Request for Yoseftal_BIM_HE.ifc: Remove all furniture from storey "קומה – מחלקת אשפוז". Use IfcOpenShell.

First a look at what the model holds.

```python
import ifcopenshell
import ifcopenshell.util.element

model = ifcopenshell.open("Yoseftal_BIM_HE.ifc")
print(model.schema)
storey = next(s for s in model.by_type("IfcBuildingStorey") if s.Name == "קומה – מחלקת אשפוז")
furniture = [e for e in ifcopenshell.util.element.get_decomposition(storey) if e.is_a("IfcFurnishingElement")]
seen = {}
for e in furniture:
    element_type = ifcopenshell.util.element.get_type(e)
    name = element_type.Name if element_type not in (None, e) else None
    seen[name] = seen.get(name, 0) + 1
for name, count in sorted(seen.items(), key=str):
    print(count, "x", name)
```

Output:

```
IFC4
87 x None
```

```python
import ifcopenshell
import ifcopenshell.api.root
import ifcopenshell.util.element

model = ifcopenshell.open("Yoseftal_BIM_HE.ifc")

storey = next(s for s in model.by_type("IfcBuildingStorey") if s.Name == "קומה – מחלקת אשפוז")
furniture = [e for e in ifcopenshell.util.element.get_decomposition(storey) if e.is_a("IfcFurnishingElement")]

for e in furniture:
    ifcopenshell.api.root.remove_product(model, product=e)
print(len(furniture), "removed")

model.write("Yoseftal_BIM_HE_updated.ifc")
```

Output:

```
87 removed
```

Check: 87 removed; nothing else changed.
